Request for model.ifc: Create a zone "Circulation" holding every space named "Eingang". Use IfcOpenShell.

First a look at what the model holds.

```python
import ifcopenshell

model = ifcopenshell.open("model.ifc")
print(model.schema)
seen = {}
for space in model.by_type("IfcSpace"):
    seen[space.LongName] = seen.get(space.LongName, 0) + 1
for name, count in sorted(seen.items(), key=str):
    print(count, "x", name)
print("zones:", [z.Name for z in model.by_type("IfcZone")][:20])
```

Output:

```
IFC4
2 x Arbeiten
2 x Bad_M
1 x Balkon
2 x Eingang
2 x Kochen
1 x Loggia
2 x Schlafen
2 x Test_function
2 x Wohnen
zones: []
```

```python
import ifcopenshell
import ifcopenshell.api.group
import ifcopenshell.api.root

model = ifcopenshell.open("model.ifc")

names = {"Eingang"}
spaces = [s for s in model.by_type("IfcSpace") if s.LongName in names]

zone = ifcopenshell.api.root.create_entity(model, ifc_class="IfcZone", name="Circulation")
ifcopenshell.api.group.assign_group(model, products=spaces, group=zone)
print(len(spaces), "spaces in", zone.Name)

model.write("model_updated.ifc")
```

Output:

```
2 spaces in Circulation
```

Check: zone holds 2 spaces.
